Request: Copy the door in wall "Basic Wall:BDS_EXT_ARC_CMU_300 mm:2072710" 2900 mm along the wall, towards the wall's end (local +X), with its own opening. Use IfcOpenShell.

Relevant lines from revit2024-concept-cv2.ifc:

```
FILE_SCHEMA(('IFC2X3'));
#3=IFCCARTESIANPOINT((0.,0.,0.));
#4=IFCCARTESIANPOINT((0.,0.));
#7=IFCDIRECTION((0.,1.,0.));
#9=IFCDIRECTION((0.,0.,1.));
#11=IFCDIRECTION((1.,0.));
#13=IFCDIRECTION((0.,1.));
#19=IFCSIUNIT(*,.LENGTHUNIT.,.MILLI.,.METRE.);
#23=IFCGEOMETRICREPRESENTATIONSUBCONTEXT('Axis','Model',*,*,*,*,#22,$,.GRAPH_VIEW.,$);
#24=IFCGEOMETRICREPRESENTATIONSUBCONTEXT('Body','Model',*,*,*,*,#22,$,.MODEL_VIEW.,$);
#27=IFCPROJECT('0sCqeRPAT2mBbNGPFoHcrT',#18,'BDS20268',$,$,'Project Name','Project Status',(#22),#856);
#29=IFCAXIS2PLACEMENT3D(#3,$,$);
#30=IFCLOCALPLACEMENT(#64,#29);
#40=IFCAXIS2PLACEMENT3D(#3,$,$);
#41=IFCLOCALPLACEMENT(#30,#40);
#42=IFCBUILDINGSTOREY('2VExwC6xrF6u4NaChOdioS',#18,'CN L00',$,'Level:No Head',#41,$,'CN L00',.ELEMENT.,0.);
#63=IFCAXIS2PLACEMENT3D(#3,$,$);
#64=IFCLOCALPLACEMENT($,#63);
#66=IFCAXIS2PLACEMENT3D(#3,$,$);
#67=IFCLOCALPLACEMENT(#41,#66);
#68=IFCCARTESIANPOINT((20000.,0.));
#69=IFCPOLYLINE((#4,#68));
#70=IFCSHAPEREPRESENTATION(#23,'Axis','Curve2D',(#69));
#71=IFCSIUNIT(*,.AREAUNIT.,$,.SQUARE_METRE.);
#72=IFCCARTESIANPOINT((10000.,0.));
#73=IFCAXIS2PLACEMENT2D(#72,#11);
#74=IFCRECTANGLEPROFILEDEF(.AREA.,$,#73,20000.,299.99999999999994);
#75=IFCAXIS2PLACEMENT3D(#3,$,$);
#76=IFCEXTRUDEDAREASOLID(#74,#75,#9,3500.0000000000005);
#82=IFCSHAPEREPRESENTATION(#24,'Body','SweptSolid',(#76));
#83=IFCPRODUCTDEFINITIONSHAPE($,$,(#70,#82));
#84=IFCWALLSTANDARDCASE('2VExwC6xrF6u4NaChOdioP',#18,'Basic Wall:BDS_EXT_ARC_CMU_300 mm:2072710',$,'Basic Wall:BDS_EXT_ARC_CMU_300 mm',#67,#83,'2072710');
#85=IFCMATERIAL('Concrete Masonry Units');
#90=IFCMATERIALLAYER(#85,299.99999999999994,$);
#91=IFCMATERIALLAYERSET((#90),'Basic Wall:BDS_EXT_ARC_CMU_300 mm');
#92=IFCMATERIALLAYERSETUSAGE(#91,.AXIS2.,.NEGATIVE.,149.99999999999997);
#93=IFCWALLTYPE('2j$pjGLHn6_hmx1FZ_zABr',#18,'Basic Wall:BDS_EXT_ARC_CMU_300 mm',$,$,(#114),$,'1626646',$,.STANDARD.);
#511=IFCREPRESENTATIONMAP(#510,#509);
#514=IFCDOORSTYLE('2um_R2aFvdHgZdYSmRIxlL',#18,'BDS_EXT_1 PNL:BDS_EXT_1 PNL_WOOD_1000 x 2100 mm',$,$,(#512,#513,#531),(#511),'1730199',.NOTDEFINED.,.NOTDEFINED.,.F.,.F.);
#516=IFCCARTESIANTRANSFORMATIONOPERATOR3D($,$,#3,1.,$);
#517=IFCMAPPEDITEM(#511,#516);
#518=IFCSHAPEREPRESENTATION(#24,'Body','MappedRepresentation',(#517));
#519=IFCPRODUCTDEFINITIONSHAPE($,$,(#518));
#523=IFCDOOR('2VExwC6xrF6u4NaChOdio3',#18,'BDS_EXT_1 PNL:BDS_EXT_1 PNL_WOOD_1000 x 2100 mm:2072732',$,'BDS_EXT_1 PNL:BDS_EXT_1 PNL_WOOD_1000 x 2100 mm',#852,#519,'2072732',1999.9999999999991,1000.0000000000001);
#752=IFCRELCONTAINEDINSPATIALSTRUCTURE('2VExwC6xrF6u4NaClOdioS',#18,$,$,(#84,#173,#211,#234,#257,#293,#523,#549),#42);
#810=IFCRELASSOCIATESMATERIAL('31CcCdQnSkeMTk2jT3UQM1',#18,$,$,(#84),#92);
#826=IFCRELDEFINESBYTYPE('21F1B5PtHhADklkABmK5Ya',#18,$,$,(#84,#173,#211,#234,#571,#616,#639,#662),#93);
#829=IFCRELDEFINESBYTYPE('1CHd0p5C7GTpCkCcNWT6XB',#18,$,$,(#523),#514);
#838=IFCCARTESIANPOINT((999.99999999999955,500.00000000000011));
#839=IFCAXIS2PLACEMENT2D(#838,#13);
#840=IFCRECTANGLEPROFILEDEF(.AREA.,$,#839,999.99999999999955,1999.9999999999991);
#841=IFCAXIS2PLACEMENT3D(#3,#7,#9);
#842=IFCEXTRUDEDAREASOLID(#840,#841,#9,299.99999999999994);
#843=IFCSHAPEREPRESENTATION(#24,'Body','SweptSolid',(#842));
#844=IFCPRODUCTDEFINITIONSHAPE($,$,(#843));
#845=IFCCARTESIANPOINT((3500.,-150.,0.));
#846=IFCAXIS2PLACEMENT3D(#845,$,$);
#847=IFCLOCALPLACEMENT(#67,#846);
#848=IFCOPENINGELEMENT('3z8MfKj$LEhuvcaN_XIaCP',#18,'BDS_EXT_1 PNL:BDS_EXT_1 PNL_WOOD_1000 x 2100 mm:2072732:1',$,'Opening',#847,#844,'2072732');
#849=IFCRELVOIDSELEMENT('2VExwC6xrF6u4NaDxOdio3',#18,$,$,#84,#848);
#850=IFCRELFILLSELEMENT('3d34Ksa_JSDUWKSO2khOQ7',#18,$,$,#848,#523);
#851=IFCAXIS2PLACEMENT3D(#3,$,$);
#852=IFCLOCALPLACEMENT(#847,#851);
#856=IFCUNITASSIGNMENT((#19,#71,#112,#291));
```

```python
import ifcopenshell
import ifcopenshell.api.feature
import ifcopenshell.api.geometry
import ifcopenshell.api.root
import ifcopenshell.geom
import ifcopenshell.util.element
import ifcopenshell.util.placement
import ifcopenshell.util.shape

model = ifcopenshell.open("revit2024-concept-cv2.ifc")
settings = ifcopenshell.geom.settings()


def volume(element):
    """Net volume in cubic metres, openings subtracted."""
    shape = ifcopenshell.geom.create_shape(settings, element)
    return ifcopenshell.util.shape.get_volume(shape.geometry)


def reuse_history(source, copy):
    """copy_class also copies each property set's owner history, people and application; keep the originals."""
    for rel in copy.IsDefinedBy:
        if rel.is_a("IfcRelDefinesByProperties") and (history := rel.RelatingPropertyDefinition.OwnerHistory):
            rel.RelatingPropertyDefinition.OwnerHistory = source.OwnerHistory
            ifcopenshell.util.element.remove_deep2(model, history)


door = model.by_id(523)
opening = door.FillsVoids[0].RelatingOpeningElement
wall = opening.VoidsElements[0].RelatingBuildingElement
before = volume(wall)
shift = ifcopenshell.util.placement.get_local_placement(wall.ObjectPlacement)[:3, 0] * 2900.0

# copy_class copies the void relationship, type, container and properties, but no geometry.
new_opening = ifcopenshell.api.root.copy_class(model, product=opening)
new_opening.Representation = ifcopenshell.util.element.copy_deep(
    model, opening.Representation, exclude=["IfcGeometricRepresentationContext", "IfcRepresentationMap"]
)
new_opening.Name = "BDS_EXT_1 PNL:BDS_EXT_1 PNL_WOOD_1000 x 2100 mm"
new_opening.Tag = None
new_door = ifcopenshell.api.root.copy_class(model, product=door)
new_door.Representation = ifcopenshell.util.element.copy_deep(
    model, door.Representation, exclude=["IfcGeometricRepresentationContext", "IfcRepresentationMap"]
)
new_door.Name = "BDS_EXT_1 PNL:BDS_EXT_1 PNL_WOOD_1000 x 2100 mm"
new_door.Tag = None
reuse_history(door, new_door)
fills = ifcopenshell.api.feature.add_filling(model, opening=new_opening, element=new_door)
fills.OwnerHistory = new_door.OwnerHistory  # required in IFC2X3

for old, new in ((opening, new_opening), (door, new_door)):
    matrix = ifcopenshell.util.placement.get_local_placement(old.ObjectPlacement)
    matrix[:3, 3] += shift
    ifcopenshell.api.geometry.edit_object_placement(model, product=new, matrix=matrix, is_si=False)

after = volume(wall)

print(f"wall volume {before:.3f} -> {after:.3f} m3")

model.write("revit2024-concept-cv2_edited.ifc")
```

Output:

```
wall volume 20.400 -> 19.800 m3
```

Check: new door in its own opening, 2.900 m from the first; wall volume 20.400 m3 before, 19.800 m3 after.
